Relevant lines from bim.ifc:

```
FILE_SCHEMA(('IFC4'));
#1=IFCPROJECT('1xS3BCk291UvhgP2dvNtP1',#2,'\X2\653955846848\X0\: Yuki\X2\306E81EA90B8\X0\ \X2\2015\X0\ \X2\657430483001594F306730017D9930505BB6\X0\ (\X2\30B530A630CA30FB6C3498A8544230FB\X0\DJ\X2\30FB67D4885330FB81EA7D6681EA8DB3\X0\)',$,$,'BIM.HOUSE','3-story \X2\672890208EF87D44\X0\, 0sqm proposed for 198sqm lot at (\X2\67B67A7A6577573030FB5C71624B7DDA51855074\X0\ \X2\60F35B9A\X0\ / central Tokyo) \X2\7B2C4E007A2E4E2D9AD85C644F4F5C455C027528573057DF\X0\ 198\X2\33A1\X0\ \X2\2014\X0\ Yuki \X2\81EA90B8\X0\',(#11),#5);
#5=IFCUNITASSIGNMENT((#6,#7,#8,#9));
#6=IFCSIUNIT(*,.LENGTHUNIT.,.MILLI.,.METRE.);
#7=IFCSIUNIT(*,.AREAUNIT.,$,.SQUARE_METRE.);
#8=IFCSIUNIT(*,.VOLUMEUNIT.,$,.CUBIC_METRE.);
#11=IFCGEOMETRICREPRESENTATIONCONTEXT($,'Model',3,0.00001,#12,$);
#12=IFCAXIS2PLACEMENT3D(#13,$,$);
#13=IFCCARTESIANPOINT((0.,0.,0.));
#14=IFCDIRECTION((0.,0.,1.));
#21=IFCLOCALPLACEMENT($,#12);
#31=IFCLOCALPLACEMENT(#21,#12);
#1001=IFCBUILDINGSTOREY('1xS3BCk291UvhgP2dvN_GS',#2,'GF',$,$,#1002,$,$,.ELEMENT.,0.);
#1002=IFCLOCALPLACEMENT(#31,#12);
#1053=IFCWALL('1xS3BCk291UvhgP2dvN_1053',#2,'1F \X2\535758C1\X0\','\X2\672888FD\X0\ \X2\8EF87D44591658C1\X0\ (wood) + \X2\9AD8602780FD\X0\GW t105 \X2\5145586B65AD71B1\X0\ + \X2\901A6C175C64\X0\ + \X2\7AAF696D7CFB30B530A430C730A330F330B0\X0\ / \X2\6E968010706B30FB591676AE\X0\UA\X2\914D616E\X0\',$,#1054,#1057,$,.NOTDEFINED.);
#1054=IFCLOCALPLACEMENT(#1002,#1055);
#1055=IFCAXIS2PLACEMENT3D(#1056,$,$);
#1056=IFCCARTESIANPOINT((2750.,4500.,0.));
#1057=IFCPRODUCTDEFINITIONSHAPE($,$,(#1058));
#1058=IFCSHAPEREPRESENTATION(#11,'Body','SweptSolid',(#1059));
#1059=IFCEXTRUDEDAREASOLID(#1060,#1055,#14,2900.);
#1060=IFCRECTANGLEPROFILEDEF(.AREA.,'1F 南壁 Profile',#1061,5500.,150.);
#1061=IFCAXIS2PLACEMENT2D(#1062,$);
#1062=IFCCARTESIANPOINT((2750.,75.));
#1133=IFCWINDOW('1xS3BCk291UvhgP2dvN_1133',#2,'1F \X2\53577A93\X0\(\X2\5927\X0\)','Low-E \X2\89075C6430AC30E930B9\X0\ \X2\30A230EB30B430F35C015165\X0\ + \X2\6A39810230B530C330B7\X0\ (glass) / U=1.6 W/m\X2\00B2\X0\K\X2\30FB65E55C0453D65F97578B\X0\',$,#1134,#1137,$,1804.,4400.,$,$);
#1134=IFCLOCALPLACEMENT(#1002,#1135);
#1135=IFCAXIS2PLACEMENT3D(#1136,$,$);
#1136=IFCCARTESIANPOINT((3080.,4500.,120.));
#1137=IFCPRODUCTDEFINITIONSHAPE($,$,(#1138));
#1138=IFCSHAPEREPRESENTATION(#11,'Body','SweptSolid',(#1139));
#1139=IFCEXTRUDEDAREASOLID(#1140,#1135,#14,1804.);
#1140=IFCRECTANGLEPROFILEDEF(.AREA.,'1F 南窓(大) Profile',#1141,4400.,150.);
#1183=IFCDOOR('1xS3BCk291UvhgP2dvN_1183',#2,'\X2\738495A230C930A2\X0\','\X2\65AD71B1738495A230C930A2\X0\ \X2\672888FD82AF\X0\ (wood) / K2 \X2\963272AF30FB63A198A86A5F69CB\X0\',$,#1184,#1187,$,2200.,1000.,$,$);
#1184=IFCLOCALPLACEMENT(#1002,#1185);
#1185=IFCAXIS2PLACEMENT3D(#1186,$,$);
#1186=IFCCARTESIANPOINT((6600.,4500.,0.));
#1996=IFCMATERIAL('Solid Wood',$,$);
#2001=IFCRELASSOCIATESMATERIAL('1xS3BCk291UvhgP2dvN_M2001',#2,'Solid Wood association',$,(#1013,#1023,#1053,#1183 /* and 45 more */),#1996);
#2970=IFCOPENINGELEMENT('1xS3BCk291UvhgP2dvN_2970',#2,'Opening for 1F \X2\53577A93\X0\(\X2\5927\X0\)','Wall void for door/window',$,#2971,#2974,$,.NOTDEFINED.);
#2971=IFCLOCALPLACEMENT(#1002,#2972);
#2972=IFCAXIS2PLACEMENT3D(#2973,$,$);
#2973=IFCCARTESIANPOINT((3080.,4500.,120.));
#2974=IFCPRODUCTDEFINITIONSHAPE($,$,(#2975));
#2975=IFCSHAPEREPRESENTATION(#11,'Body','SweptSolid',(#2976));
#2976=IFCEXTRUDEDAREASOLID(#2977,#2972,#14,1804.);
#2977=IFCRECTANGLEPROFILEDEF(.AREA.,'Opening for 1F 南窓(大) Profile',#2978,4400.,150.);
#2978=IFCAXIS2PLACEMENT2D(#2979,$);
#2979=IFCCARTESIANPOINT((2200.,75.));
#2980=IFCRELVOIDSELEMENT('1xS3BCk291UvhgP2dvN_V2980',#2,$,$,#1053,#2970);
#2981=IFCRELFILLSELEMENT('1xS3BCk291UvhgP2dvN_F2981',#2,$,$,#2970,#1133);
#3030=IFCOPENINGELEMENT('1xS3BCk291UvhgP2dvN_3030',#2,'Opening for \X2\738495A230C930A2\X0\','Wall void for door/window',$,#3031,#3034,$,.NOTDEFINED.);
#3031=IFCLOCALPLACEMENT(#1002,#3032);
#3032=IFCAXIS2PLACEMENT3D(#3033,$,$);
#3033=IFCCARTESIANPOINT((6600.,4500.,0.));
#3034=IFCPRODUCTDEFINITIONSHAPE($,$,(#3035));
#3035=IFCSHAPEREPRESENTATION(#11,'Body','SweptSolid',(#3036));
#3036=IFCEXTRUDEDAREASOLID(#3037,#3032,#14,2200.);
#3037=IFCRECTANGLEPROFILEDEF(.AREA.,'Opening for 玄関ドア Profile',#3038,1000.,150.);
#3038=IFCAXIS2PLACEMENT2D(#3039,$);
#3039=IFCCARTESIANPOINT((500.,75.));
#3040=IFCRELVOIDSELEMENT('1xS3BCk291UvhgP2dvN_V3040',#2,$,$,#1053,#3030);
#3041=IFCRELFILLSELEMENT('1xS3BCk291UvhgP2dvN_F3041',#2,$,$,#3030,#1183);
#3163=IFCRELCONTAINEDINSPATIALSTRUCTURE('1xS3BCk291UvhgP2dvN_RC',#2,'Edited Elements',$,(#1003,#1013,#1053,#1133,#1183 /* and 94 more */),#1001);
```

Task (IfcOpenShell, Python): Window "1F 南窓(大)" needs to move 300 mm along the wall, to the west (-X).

```python
import ifcopenshell
import ifcopenshell.api.geometry
import ifcopenshell.util.placement
import ifcopenshell.util.unit

model = ifcopenshell.open("bim.ifc")
unit_scale = ifcopenshell.util.unit.calculate_unit_scale(model)

window = model.by_guid("1xS3BCk291UvhgP2dvN_1133")
opening = window.FillsVoids[0].RelatingOpeningElement
wall = opening.VoidsElements[0].RelatingBuildingElement

wall_matrix = ifcopenshell.util.placement.get_local_placement(wall.ObjectPlacement)
shift = wall_matrix[:3, 0] * -0.3 / unit_scale
before = ifcopenshell.util.placement.get_local_placement(window.ObjectPlacement)[:3, 3].copy()

# The window is not placed relative to its opening, so move both.
for product in (opening, window):
    matrix = ifcopenshell.util.placement.get_local_placement(product.ObjectPlacement)
    matrix[:3, 3] += shift
    ifcopenshell.api.geometry.edit_object_placement(model, product=product, matrix=matrix, is_si=False)

after = ifcopenshell.util.placement.get_local_placement(window.ObjectPlacement)[:3, 3]
print("window moved by", (after - before).round(3) + 0.0)

model.write("bim-out.ifc")
```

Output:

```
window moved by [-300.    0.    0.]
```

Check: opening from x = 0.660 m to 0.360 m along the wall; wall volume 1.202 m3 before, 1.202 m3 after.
